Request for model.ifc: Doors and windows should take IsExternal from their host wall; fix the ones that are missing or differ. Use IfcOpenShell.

First a look at what the model holds.

```python
import ifcopenshell
import ifcopenshell.util.element

model = ifcopenshell.open("model.ifc")
print(model.schema)
seen = {}
for e in model.by_type("IfcDoor") + model.by_type("IfcWindow"):
    if not e.FillsVoids:
        continue
    host = e.FillsVoids[0].RelatingOpeningElement.VoidsElements[0].RelatingBuildingElement
    own = ifcopenshell.util.element.get_pset(e, f"Pset_{e.is_a()[3:].removesuffix('StandardCase')}Common", "IsExternal")
    wall = ifcopenshell.util.element.get_pset(host, "Pset_WallCommon", "IsExternal")
    seen[e.is_a(), own, wall] = seen.get((e.is_a(), own, wall), 0) + 1
for (cls, own, wall), count in sorted(seen.items(), key=str):
    print(count, cls, "IsExternal:", own, "| host wall:", wall)
```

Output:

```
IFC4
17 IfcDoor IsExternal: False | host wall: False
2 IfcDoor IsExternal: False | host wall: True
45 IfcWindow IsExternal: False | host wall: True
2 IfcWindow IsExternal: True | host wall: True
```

```python
import ifcopenshell
import ifcopenshell.api.pset
import ifcopenshell.util.element

model = ifcopenshell.open("model.ifc")

count = 0
for ifc_class, pset_name in (("IfcDoor", "Pset_DoorCommon"), ("IfcWindow", "Pset_WindowCommon")):
    for e in model.by_type(ifc_class):
        if not e.FillsVoids:
            continue
        host = e.FillsVoids[0].RelatingOpeningElement.VoidsElements[0].RelatingBuildingElement
        external = ifcopenshell.util.element.get_pset(host, "Pset_WallCommon", "IsExternal")
        if external is None or ifcopenshell.util.element.get_pset(e, pset_name, "IsExternal") == external:
            continue
        pset = ifcopenshell.api.pset.add_pset(model, product=e, name=pset_name)
        ifcopenshell.api.pset.edit_pset(model, pset=pset, properties={"IsExternal": external})
        count += 1

print(count, "updated")

model.write("model_v2.ifc")
```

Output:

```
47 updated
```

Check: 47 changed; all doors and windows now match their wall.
